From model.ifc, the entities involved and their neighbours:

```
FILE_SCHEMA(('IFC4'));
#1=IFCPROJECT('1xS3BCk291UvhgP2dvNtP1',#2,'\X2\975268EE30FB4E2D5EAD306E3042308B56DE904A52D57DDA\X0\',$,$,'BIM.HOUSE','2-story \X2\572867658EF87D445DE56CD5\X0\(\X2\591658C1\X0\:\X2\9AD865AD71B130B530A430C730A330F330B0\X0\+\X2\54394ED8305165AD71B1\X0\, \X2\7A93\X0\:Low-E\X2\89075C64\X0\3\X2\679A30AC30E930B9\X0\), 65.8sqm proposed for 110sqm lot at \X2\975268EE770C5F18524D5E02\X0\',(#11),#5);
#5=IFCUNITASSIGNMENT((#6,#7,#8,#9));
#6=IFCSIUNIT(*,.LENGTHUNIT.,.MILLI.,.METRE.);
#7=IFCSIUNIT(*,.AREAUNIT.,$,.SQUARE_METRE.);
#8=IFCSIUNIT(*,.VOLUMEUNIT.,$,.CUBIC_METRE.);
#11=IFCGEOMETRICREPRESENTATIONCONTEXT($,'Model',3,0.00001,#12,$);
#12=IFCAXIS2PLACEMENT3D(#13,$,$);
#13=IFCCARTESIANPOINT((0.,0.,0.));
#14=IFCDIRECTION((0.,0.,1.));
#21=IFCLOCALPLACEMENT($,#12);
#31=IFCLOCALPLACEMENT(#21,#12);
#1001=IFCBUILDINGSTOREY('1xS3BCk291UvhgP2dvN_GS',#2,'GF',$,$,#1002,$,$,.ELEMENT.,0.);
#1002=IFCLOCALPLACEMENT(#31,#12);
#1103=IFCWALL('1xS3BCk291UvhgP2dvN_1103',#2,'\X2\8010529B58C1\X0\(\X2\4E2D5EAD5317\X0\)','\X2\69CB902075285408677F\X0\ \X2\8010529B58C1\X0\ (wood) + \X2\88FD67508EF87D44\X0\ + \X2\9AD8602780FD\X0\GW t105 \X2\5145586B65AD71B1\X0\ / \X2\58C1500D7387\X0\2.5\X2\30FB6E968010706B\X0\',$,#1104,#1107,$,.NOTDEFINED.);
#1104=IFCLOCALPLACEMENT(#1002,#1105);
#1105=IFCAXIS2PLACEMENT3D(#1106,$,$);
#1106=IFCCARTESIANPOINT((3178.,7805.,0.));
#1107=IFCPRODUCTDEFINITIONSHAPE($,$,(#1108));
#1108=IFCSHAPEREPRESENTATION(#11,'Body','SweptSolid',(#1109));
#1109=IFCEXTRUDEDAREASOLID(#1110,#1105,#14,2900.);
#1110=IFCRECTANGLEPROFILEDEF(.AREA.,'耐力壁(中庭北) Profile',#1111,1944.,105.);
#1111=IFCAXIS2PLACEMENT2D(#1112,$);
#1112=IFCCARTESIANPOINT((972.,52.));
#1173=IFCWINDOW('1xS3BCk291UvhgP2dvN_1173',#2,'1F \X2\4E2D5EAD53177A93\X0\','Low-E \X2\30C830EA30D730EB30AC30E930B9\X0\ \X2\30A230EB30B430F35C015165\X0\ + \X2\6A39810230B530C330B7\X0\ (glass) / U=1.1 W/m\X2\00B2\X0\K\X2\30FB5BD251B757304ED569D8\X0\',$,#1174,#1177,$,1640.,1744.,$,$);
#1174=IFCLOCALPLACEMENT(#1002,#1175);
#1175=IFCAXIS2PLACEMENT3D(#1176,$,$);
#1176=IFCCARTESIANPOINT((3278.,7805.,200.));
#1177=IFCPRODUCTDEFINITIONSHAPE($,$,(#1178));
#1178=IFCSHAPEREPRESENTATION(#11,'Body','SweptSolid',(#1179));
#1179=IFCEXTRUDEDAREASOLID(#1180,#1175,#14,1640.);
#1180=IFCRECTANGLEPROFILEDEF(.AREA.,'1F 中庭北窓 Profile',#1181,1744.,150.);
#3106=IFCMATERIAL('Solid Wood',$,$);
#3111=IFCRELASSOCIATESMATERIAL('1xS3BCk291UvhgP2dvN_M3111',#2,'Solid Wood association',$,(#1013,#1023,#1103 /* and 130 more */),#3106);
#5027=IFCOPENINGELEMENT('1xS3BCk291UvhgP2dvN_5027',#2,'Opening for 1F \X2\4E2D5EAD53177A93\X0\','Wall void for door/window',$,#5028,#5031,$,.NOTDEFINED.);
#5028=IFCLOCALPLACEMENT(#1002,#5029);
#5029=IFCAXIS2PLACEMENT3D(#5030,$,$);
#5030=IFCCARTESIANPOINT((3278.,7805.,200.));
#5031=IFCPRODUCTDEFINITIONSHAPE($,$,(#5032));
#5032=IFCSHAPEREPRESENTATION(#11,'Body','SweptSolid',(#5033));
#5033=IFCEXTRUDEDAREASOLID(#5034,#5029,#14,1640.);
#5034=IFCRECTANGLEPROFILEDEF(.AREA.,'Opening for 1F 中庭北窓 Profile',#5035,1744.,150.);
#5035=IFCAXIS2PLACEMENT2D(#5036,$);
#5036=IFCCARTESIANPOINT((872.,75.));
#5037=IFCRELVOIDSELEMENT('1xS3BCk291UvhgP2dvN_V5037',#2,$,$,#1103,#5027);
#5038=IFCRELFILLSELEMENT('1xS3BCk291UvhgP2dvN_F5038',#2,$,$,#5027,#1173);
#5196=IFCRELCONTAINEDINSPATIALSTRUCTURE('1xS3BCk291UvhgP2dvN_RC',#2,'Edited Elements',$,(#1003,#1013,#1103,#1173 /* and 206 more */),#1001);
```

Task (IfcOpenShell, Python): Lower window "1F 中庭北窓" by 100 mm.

```python
import numpy as np
import ifcopenshell
import ifcopenshell.api.geometry
import ifcopenshell.util.placement
import ifcopenshell.util.unit

model = ifcopenshell.open("model.ifc")
unit_scale = ifcopenshell.util.unit.calculate_unit_scale(model)

window = model.by_guid("1xS3BCk291UvhgP2dvN_1173")
opening = window.FillsVoids[0].RelatingOpeningElement
dz = -100.0

shift = np.array([0.0, 0.0, dz])
# The window is not placed relative to its opening, so move both.
for product in (opening, window):
    matrix = ifcopenshell.util.placement.get_local_placement(product.ObjectPlacement)
    matrix[:3, 3] += shift
    ifcopenshell.api.geometry.edit_object_placement(model, product=product, matrix=matrix, is_si=False)

print(f"moved by {dz * unit_scale:+.3f} m")

model.write("model_v2.ifc")
```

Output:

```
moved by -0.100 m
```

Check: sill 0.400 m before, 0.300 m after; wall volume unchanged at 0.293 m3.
